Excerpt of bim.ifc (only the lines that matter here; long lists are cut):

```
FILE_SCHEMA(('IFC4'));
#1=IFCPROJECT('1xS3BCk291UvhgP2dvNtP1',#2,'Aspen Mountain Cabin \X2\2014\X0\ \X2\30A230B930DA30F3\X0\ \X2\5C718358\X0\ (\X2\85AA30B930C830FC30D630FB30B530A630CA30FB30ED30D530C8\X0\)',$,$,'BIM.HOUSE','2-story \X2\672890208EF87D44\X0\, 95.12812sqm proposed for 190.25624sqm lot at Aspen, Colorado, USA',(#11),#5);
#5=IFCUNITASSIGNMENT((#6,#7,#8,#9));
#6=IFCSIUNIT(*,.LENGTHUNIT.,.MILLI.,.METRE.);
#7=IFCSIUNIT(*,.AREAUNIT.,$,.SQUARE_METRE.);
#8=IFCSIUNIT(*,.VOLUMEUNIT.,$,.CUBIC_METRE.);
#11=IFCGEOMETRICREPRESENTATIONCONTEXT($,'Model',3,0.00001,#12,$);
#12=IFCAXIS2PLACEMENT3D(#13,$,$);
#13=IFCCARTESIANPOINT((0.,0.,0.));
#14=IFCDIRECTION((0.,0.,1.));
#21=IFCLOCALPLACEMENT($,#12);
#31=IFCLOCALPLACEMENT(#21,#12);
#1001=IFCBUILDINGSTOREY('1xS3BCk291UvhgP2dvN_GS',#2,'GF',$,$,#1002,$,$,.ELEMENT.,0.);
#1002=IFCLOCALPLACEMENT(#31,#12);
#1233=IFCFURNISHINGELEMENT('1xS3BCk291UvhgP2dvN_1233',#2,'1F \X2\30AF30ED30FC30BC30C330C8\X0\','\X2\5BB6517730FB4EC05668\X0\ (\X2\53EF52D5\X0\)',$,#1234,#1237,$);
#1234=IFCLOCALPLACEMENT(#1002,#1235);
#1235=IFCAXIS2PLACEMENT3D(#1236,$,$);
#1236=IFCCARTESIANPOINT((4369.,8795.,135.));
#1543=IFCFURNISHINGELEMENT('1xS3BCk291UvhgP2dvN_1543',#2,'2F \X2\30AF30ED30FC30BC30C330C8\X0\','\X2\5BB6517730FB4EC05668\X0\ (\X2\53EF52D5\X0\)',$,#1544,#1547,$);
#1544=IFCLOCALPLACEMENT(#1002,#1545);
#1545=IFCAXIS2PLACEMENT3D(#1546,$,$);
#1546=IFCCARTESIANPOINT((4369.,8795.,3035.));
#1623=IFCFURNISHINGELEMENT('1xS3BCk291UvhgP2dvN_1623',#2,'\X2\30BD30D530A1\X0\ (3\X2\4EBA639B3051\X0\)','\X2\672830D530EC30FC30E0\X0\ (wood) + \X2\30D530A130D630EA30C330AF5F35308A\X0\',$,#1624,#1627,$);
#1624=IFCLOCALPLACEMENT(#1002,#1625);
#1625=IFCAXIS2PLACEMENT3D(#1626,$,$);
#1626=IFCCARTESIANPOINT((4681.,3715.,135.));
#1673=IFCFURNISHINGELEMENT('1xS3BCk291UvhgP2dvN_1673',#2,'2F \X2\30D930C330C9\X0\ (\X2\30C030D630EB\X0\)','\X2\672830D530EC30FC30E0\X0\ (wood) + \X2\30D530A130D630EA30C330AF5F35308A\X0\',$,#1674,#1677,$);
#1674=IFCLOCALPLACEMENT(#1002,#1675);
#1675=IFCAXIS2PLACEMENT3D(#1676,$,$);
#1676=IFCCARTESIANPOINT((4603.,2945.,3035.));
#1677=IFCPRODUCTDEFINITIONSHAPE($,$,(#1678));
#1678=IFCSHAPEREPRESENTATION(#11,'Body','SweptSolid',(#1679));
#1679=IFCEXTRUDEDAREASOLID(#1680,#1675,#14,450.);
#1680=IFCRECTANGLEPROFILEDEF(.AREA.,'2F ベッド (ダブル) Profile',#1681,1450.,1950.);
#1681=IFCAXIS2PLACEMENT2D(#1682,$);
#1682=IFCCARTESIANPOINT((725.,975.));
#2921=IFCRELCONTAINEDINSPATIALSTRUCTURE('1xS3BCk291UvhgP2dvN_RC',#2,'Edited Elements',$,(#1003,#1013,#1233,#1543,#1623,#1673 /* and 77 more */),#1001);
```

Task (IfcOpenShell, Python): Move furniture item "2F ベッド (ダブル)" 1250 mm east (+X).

```python
import ifcopenshell
import ifcopenshell.api.geometry
import ifcopenshell.util.placement
import ifcopenshell.util.unit

model = ifcopenshell.open("bim.ifc")
unit_scale = ifcopenshell.util.unit.calculate_unit_scale(model)

item = model.by_guid("1xS3BCk291UvhgP2dvN_1673")
matrix = ifcopenshell.util.placement.get_local_placement(item.ObjectPlacement)
matrix[0, 3] += 1.25 / unit_scale
ifcopenshell.api.geometry.edit_object_placement(model, product=item, matrix=matrix, is_si=False)

print(ifcopenshell.util.placement.get_local_placement(item.ObjectPlacement).round(3) + 0.0)

model.write("bim_v2.ifc")
```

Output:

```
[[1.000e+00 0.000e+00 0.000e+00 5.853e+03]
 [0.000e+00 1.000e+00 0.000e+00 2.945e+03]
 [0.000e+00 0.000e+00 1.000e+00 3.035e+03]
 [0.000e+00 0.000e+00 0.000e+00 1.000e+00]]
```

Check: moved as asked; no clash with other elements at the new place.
